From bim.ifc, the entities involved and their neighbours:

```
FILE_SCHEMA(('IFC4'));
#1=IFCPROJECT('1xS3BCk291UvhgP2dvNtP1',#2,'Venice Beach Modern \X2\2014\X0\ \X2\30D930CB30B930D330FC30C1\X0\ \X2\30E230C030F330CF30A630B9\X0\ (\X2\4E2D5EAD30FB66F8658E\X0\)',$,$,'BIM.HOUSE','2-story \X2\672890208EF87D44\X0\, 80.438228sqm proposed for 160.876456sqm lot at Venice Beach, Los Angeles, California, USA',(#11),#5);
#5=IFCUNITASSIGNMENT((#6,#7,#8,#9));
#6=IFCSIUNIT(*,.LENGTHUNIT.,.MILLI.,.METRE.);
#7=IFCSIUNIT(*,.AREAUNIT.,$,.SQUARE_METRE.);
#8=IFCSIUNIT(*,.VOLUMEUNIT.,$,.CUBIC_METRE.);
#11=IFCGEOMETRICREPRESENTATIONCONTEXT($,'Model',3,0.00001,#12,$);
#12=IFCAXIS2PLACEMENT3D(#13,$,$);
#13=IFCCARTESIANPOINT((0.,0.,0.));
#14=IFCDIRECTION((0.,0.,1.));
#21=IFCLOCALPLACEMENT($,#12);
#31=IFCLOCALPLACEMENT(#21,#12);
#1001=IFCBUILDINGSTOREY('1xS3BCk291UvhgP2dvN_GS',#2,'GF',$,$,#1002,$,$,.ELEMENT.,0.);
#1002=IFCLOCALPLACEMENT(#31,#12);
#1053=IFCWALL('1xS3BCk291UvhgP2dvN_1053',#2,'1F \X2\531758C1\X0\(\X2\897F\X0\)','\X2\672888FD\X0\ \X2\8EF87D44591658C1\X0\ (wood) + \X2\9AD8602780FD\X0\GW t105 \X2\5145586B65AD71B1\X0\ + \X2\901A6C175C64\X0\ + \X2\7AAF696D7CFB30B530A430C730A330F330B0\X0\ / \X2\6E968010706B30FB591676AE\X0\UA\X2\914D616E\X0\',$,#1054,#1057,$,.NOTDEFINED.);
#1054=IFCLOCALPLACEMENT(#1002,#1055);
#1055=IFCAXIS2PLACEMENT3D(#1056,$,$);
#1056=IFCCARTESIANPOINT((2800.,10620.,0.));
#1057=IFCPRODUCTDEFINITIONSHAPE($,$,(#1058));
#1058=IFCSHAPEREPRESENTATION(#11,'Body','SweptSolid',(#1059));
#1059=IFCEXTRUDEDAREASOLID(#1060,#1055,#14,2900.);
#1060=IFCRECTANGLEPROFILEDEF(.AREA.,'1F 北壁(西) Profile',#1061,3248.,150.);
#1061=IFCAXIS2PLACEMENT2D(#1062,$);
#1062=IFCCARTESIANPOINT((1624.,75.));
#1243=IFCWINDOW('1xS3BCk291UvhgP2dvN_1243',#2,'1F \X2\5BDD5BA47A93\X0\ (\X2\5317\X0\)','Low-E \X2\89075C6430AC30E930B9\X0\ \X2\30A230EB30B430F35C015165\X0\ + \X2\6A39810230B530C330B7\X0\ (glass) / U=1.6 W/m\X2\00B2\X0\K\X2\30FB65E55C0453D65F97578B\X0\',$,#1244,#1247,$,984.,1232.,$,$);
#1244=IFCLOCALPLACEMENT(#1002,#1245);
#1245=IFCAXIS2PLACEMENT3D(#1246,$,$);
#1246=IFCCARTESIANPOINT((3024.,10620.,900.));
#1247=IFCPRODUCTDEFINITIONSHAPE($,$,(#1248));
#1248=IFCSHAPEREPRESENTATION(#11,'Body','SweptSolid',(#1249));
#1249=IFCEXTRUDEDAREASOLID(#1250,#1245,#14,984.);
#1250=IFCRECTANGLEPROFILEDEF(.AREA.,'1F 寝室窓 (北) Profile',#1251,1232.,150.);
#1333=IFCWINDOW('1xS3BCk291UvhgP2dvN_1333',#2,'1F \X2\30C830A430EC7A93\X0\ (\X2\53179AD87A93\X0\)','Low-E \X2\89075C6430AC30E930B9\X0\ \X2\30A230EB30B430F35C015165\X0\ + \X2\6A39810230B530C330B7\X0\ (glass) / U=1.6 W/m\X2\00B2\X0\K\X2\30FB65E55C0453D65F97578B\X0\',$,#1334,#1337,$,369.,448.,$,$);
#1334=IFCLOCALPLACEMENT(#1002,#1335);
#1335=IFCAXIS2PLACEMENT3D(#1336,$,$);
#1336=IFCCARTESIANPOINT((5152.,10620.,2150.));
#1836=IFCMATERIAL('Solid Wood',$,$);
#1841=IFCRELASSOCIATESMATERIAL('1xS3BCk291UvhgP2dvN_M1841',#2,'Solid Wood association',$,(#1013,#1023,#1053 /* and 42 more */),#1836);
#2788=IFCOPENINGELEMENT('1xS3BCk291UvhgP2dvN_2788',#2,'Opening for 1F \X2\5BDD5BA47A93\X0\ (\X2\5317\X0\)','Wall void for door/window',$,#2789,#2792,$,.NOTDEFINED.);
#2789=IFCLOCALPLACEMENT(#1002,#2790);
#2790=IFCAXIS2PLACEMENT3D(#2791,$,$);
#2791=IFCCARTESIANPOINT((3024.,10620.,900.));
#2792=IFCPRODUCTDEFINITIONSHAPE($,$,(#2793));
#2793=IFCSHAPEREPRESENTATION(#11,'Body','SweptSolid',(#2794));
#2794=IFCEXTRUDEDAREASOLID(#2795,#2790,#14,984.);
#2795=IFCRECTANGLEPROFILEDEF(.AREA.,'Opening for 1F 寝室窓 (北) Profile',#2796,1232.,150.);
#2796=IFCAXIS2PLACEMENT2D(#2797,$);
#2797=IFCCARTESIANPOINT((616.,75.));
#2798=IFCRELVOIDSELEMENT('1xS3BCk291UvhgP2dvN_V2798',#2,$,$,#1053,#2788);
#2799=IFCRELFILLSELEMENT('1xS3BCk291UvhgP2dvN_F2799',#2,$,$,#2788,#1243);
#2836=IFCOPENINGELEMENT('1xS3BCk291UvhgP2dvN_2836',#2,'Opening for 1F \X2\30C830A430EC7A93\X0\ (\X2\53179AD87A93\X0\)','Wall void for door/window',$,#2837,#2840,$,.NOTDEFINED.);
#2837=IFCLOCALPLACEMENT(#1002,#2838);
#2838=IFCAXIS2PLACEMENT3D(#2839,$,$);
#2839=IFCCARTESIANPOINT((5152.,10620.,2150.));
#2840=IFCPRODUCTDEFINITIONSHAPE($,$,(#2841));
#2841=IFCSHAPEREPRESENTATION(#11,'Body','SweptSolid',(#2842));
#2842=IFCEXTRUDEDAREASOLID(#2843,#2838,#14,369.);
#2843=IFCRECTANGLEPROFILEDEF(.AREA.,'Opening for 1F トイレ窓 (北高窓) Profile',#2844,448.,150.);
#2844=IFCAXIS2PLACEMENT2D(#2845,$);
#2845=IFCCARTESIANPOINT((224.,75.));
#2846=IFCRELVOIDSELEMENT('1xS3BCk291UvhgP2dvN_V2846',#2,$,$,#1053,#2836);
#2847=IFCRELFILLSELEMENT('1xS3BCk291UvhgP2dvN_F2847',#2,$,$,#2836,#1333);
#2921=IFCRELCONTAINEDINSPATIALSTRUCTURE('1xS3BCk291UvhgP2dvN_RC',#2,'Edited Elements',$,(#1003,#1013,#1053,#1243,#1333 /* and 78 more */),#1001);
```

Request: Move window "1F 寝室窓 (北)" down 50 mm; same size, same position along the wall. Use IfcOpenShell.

```python
import numpy as np
import ifcopenshell
import ifcopenshell.api.geometry
import ifcopenshell.util.placement
import ifcopenshell.util.unit

model = ifcopenshell.open("bim.ifc")
unit_scale = ifcopenshell.util.unit.calculate_unit_scale(model)

window = model.by_guid("1xS3BCk291UvhgP2dvN_1243")
opening = window.FillsVoids[0].RelatingOpeningElement
dz = -0.05 / unit_scale

shift = np.array([0.0, 0.0, dz])
# The window is not placed relative to its opening, so move both.
for product in (opening, window):
    matrix = ifcopenshell.util.placement.get_local_placement(product.ObjectPlacement)
    matrix[:3, 3] += shift
    ifcopenshell.api.geometry.edit_object_placement(model, product=product, matrix=matrix, is_si=False)

print(f"moved by {dz * unit_scale:+.3f} m")

model.write("bim_edited.ifc")
```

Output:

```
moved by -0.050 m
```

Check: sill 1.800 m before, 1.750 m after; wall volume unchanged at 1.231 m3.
